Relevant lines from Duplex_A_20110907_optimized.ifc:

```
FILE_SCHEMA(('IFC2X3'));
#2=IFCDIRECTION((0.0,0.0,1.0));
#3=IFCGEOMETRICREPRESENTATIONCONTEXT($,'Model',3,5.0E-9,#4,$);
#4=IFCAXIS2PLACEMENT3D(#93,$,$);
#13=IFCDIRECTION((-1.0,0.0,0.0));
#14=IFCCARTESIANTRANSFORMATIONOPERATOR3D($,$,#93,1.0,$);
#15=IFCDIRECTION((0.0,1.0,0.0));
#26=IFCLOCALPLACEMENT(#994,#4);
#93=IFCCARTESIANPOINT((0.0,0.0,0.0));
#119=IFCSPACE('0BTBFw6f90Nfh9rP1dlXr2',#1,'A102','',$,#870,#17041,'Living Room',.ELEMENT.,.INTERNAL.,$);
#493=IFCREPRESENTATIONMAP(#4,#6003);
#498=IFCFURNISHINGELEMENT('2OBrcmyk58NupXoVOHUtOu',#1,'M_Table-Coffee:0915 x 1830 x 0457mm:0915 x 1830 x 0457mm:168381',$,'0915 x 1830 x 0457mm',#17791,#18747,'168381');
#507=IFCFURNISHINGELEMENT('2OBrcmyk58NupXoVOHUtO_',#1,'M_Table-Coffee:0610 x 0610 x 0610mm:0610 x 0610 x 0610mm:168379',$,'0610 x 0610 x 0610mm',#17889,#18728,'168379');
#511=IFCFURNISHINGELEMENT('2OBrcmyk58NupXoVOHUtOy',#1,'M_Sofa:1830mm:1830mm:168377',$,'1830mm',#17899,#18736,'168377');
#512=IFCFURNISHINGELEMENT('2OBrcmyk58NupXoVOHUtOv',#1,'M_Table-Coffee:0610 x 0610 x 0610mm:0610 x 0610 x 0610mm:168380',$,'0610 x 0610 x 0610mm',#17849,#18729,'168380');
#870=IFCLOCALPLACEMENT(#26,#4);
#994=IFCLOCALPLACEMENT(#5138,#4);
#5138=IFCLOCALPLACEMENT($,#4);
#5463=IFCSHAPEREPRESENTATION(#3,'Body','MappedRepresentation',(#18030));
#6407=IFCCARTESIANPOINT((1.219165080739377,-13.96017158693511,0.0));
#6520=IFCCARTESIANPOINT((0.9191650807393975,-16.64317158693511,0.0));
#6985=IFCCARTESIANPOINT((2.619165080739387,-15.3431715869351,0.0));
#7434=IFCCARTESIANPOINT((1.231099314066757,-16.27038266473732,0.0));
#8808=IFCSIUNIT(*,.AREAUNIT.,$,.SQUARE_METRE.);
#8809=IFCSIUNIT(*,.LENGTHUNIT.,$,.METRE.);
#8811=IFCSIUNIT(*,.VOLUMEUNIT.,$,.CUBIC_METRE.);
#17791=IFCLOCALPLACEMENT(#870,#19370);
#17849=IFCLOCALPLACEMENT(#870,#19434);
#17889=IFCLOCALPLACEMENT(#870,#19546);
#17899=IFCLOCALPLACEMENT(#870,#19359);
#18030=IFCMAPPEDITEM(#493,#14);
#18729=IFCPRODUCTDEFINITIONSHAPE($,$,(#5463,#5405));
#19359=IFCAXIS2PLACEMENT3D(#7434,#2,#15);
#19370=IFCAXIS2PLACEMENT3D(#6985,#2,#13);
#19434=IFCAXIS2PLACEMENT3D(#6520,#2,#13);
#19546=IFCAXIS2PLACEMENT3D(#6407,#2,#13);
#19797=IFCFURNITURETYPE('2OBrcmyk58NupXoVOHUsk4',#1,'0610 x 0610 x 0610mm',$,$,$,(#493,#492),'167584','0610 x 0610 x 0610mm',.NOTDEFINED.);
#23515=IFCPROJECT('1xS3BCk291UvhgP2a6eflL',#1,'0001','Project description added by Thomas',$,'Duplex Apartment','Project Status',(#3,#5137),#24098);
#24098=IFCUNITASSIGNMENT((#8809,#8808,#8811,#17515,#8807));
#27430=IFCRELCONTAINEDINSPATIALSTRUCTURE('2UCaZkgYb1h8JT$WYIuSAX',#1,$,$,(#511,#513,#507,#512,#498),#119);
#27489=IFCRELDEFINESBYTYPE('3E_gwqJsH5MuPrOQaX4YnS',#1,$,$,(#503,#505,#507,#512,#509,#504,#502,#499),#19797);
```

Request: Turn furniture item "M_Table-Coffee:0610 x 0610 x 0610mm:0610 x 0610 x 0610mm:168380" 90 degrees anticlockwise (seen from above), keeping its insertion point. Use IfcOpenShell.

```python
import ifcopenshell
import ifcopenshell.api.geometry
import ifcopenshell.util.placement

model = ifcopenshell.open("Duplex_A_20110907_optimized.ifc")

item = model.by_id(512)
matrix = ifcopenshell.util.placement.get_local_placement(item.ObjectPlacement)
matrix = matrix @ ifcopenshell.util.placement.rotation(90, "Z")
ifcopenshell.api.geometry.edit_object_placement(model, product=item, matrix=matrix, is_si=False)

print(ifcopenshell.util.placement.get_local_placement(item.ObjectPlacement).round(3) + 0.0)

model.write("Duplex_A_20110907_optimized-out.ifc")
```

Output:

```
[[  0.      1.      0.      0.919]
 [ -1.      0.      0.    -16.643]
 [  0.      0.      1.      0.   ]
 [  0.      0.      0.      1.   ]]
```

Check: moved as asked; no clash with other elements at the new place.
